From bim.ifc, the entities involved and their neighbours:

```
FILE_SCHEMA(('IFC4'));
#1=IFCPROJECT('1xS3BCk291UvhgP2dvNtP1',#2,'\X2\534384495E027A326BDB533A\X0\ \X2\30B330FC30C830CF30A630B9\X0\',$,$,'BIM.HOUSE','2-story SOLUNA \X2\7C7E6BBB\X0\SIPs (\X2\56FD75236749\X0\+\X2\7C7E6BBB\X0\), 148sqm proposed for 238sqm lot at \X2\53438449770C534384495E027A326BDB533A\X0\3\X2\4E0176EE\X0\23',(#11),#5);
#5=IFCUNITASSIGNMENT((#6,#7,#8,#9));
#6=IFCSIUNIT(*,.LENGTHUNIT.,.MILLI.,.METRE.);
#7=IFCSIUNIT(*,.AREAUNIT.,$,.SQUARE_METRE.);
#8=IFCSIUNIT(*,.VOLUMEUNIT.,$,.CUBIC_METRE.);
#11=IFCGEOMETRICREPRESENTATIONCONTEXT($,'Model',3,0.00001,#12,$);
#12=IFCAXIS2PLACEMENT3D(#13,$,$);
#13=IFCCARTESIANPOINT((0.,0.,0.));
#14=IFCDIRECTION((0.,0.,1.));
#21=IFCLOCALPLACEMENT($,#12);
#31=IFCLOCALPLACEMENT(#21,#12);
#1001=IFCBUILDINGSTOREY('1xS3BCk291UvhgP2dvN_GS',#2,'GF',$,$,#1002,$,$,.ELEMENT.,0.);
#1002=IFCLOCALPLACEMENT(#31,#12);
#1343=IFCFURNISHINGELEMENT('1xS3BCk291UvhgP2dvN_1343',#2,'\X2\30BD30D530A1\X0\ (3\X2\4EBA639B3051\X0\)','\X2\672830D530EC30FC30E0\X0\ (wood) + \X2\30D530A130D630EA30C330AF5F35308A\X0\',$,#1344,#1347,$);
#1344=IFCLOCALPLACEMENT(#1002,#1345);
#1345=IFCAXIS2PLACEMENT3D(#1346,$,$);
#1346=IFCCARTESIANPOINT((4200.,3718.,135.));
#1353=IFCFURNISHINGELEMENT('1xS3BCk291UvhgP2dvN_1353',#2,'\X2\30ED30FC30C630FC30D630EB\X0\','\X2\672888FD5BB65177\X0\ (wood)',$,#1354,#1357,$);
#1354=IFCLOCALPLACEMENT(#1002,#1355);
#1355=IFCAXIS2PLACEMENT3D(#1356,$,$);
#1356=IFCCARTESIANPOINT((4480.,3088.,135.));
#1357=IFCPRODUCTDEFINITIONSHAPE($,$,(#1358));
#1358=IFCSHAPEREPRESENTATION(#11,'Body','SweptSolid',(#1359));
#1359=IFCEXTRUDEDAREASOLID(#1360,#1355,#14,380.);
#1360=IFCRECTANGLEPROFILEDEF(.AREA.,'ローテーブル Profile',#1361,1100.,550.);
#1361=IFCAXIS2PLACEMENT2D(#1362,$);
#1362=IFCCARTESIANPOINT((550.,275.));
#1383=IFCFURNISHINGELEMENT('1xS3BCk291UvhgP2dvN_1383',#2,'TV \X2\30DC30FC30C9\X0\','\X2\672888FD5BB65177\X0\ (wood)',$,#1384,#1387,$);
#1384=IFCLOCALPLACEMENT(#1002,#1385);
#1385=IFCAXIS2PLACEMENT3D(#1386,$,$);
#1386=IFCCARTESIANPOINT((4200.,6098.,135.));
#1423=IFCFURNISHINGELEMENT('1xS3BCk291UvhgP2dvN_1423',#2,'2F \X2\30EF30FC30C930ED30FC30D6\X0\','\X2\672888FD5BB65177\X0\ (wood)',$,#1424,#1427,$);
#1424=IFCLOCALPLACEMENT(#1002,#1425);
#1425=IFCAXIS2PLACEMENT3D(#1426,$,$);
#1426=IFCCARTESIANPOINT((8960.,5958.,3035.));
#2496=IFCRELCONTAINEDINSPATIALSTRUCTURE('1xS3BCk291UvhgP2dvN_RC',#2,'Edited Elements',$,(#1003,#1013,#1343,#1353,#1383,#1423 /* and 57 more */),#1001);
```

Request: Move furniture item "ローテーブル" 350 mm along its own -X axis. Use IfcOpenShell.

```python
import ifcopenshell
import ifcopenshell.api.geometry
import ifcopenshell.util.placement
import ifcopenshell.util.unit

model = ifcopenshell.open("bim.ifc")
unit_scale = ifcopenshell.util.unit.calculate_unit_scale(model)

item = model.by_guid("1xS3BCk291UvhgP2dvN_1353")
matrix = ifcopenshell.util.placement.get_local_placement(item.ObjectPlacement)
matrix[:3, 3] -= matrix[:3, 0] * 0.35 / unit_scale
ifcopenshell.api.geometry.edit_object_placement(model, product=item, matrix=matrix, is_si=False)

print(ifcopenshell.util.placement.get_local_placement(item.ObjectPlacement).round(3) + 0.0)

model.write("bim_rev.ifc")
```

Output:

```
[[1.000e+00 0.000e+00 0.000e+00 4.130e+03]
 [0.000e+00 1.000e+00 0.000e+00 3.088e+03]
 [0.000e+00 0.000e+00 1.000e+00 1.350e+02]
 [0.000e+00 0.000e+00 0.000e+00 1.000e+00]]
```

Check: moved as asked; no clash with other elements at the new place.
